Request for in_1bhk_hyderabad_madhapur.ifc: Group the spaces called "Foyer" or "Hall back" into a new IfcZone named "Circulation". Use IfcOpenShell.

First a look at what the model holds.

```python
import ifcopenshell

model = ifcopenshell.open("in_1bhk_hyderabad_madhapur.ifc")
print(model.schema)
seen = {}
for space in model.by_type("IfcSpace"):
    seen[space.LongName] = seen.get(space.LongName, 0) + 1
for name, count in sorted(seen.items(), key=str):
    print(count, "x", name)
print("zones:", [z.Name for z in model.by_type("IfcZone")][:20])
```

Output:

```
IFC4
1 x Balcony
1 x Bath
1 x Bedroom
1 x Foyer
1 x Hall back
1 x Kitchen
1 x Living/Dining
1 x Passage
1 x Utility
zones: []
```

```python
import ifcopenshell
import ifcopenshell.api.group
import ifcopenshell.api.root

model = ifcopenshell.open("in_1bhk_hyderabad_madhapur.ifc")

names = {"Foyer", "Hall back"}
spaces = [s for s in model.by_type("IfcSpace") if s.LongName in names]

zone = ifcopenshell.api.root.create_entity(model, ifc_class="IfcZone", name="Circulation")
ifcopenshell.api.group.assign_group(model, products=spaces, group=zone)
print(len(spaces), "spaces in", zone.Name)

model.write("in_1bhk_hyderabad_madhapur-out.ifc")
```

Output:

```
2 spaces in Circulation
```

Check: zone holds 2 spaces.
